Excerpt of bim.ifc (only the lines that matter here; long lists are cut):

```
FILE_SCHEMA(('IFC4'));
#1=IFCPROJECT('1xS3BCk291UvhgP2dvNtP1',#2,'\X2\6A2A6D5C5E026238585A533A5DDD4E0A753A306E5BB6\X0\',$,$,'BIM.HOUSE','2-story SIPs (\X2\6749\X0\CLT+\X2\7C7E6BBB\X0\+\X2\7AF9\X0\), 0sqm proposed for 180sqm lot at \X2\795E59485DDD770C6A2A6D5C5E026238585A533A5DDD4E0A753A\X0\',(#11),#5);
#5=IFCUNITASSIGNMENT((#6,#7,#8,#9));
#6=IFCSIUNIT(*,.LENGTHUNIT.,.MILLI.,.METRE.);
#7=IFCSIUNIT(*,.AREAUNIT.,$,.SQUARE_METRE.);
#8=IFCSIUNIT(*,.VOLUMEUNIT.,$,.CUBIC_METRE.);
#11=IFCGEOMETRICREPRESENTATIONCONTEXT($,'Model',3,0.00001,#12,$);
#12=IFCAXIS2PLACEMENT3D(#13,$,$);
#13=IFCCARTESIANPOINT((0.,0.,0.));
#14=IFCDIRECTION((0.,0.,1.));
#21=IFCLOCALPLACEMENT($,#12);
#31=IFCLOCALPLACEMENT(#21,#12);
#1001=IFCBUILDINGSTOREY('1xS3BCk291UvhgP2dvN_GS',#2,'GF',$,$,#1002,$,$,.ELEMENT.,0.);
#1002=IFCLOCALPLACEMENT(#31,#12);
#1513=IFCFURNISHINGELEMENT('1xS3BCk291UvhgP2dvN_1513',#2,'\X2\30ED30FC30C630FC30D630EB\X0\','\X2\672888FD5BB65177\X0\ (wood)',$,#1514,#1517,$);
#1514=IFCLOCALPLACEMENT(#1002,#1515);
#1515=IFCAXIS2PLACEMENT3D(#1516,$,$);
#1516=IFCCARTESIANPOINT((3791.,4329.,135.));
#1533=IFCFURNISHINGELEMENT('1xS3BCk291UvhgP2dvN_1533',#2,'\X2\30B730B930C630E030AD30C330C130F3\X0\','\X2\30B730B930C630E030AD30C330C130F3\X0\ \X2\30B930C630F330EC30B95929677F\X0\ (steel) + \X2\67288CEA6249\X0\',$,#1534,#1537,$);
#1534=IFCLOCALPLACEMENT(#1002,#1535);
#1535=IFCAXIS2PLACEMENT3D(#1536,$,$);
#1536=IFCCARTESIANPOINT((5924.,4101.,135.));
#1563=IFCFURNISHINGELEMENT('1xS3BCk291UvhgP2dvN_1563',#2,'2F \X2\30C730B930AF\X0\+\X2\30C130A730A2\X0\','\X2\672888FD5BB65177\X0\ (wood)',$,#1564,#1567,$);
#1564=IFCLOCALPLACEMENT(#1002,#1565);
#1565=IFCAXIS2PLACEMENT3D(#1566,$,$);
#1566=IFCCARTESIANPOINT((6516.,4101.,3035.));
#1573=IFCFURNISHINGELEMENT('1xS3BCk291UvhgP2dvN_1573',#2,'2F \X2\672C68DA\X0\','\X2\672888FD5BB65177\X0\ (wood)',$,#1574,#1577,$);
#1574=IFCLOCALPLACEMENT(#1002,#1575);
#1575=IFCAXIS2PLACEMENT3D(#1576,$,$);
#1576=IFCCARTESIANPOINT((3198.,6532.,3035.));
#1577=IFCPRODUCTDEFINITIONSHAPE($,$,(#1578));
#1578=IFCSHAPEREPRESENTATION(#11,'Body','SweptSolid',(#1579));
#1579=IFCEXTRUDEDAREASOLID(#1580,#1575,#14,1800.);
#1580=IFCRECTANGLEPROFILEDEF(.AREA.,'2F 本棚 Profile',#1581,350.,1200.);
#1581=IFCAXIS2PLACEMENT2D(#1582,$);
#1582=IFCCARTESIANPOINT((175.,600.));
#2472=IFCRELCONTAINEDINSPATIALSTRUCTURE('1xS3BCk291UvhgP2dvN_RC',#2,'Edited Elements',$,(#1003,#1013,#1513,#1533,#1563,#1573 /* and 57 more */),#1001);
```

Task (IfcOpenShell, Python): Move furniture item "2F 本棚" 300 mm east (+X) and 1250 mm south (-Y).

```python
import ifcopenshell
import ifcopenshell.api.geometry
import ifcopenshell.util.placement
import ifcopenshell.util.unit

model = ifcopenshell.open("bim.ifc")
unit_scale = ifcopenshell.util.unit.calculate_unit_scale(model)

item = model.by_guid("1xS3BCk291UvhgP2dvN_1573")
matrix = ifcopenshell.util.placement.get_local_placement(item.ObjectPlacement)
matrix[0, 3] += 0.3 / unit_scale
matrix[1, 3] -= 1.25 / unit_scale
ifcopenshell.api.geometry.edit_object_placement(model, product=item, matrix=matrix, is_si=False)

print(ifcopenshell.util.placement.get_local_placement(item.ObjectPlacement).round(3) + 0.0)

model.write("bim_rev.ifc")
```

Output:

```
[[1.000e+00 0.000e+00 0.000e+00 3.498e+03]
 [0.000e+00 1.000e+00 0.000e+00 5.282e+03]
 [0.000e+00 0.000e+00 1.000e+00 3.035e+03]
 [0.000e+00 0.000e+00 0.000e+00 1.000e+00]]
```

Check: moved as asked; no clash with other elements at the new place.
